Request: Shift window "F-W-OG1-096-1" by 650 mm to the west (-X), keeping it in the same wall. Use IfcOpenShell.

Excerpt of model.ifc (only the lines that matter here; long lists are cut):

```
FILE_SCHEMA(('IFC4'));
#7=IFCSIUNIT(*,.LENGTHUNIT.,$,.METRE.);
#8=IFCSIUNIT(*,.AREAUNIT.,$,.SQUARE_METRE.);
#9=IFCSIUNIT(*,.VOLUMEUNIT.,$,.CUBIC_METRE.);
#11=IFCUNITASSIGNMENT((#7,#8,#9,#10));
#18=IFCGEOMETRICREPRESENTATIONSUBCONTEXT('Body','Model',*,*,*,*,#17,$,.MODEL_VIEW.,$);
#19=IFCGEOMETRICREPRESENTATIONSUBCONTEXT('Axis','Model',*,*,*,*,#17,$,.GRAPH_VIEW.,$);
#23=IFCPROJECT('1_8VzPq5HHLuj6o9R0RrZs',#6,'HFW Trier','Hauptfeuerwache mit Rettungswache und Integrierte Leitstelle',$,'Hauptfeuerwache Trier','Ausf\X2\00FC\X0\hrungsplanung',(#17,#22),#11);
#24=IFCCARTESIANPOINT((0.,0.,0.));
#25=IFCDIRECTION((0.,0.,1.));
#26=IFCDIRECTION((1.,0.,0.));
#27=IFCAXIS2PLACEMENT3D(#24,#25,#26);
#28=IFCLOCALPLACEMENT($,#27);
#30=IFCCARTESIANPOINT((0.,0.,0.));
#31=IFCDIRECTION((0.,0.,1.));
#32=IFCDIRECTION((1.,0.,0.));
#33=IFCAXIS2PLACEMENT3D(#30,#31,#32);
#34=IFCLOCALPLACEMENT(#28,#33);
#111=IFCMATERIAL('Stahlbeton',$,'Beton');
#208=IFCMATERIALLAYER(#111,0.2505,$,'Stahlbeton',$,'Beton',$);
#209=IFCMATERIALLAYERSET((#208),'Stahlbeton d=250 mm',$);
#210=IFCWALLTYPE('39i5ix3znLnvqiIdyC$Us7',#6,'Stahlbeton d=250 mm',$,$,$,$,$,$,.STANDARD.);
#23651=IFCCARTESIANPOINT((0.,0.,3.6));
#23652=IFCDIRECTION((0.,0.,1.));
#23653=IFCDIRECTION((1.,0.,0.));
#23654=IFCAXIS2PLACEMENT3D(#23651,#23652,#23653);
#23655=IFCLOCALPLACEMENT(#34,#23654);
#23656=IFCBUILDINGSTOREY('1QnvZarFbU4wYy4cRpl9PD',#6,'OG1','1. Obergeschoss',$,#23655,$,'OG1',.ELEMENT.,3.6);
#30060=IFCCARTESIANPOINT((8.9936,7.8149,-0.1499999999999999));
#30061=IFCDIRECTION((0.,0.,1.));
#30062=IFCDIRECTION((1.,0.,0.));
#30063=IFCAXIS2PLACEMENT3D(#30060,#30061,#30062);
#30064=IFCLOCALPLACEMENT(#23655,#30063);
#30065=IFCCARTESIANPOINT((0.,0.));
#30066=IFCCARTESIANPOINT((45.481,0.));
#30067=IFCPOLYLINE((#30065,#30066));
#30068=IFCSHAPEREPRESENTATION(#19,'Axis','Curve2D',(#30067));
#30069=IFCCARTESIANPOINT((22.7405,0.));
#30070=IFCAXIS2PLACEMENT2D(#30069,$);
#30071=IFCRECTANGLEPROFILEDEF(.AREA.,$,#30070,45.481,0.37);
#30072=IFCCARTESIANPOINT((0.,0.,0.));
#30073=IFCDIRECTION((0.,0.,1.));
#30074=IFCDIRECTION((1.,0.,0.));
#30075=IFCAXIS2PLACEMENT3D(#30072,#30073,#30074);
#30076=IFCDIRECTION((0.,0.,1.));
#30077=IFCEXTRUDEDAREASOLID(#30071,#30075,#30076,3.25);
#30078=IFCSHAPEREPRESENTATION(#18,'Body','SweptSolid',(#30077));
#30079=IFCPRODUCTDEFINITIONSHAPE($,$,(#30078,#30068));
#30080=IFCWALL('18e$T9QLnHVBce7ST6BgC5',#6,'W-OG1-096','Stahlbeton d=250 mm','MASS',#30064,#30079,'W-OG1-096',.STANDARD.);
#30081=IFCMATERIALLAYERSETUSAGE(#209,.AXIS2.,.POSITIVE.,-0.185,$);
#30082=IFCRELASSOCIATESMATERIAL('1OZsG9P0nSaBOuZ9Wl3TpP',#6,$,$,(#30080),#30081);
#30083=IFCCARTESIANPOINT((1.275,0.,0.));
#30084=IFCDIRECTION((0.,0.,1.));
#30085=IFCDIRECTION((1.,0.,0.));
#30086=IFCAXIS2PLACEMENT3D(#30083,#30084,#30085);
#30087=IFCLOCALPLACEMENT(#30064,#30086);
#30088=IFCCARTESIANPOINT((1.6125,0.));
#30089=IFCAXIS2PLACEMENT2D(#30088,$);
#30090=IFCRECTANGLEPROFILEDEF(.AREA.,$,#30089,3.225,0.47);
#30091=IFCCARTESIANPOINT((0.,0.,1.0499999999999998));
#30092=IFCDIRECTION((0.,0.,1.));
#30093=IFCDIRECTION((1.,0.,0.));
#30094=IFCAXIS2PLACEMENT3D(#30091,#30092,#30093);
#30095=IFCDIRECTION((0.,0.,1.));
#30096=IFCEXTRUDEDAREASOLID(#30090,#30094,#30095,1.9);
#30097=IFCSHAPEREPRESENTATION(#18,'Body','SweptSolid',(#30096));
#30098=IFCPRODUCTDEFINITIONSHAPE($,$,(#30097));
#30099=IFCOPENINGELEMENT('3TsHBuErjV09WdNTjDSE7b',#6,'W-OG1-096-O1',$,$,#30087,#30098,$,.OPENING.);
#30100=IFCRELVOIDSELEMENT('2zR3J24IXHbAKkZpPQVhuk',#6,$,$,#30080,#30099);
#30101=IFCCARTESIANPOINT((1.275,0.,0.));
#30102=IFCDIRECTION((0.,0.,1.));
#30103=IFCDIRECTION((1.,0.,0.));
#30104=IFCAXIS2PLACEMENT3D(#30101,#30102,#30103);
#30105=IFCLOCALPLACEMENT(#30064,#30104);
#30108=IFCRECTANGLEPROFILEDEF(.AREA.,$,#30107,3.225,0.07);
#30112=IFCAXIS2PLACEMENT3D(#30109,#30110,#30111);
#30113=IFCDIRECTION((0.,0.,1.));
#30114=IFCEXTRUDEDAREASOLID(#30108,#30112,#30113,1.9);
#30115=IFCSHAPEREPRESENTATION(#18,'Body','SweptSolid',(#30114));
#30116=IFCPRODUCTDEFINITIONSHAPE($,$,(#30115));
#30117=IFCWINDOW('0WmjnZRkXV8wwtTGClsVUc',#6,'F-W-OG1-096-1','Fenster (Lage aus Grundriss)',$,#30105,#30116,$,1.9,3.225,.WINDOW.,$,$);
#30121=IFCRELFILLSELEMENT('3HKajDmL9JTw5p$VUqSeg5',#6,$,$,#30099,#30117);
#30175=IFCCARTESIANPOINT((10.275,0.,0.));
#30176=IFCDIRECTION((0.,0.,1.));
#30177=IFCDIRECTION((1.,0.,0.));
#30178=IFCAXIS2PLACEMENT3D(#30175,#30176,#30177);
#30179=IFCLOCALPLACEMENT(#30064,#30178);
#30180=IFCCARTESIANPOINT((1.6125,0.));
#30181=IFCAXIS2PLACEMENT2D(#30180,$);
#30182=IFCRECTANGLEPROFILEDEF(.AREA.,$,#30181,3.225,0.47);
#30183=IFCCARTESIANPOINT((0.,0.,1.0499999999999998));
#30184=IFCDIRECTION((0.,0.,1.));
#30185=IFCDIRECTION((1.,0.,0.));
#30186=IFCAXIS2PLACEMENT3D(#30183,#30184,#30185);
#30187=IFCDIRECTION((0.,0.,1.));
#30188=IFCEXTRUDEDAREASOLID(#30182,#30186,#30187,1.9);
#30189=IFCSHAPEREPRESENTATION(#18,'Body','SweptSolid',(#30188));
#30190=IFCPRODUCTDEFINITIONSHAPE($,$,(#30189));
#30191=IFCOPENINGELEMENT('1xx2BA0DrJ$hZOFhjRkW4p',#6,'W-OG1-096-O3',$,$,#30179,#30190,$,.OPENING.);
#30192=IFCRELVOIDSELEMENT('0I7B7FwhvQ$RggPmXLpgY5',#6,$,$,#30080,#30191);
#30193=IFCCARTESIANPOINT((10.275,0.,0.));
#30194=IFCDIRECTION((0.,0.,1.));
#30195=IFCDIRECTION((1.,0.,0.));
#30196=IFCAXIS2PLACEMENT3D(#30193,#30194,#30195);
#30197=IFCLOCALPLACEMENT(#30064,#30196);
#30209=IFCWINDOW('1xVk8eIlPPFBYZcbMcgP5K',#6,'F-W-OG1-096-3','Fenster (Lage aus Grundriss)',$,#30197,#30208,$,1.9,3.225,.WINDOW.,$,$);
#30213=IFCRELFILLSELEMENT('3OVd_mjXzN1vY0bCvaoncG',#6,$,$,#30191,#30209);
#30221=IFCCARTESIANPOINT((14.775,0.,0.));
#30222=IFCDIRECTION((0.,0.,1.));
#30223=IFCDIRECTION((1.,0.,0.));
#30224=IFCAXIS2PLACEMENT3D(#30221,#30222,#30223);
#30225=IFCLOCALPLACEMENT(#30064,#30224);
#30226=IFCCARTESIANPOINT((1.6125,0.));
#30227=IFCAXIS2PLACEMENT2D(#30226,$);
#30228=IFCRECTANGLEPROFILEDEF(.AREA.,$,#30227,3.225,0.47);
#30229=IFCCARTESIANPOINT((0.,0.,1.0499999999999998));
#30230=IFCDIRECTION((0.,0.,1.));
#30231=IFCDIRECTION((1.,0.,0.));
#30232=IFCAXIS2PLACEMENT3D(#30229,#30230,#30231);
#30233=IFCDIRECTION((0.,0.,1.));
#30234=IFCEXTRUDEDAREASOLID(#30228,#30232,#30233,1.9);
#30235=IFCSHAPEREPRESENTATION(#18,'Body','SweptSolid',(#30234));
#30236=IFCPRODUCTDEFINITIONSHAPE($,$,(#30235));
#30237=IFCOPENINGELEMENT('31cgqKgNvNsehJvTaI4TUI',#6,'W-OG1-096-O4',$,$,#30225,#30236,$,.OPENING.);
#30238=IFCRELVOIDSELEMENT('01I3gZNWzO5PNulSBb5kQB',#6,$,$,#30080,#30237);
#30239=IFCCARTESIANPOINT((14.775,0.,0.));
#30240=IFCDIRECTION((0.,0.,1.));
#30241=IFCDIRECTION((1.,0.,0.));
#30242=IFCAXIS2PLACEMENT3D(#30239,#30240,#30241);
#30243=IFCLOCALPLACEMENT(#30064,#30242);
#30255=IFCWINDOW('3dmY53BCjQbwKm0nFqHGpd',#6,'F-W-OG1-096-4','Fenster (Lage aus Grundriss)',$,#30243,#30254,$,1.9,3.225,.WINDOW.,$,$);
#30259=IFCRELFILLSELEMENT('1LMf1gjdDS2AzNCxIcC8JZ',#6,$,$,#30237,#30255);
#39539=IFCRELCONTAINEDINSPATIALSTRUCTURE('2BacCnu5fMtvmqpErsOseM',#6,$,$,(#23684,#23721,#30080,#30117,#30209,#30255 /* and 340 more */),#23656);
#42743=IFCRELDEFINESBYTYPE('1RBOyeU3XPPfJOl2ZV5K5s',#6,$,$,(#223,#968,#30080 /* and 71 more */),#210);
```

```python
import ifcopenshell
import ifcopenshell.api.geometry
import ifcopenshell.util.placement
import ifcopenshell.util.unit

model = ifcopenshell.open("model.ifc")
unit_scale = ifcopenshell.util.unit.calculate_unit_scale(model)

window = model.by_guid("0WmjnZRkXV8wwtTGClsVUc")
opening = window.FillsVoids[0].RelatingOpeningElement
wall = opening.VoidsElements[0].RelatingBuildingElement

wall_matrix = ifcopenshell.util.placement.get_local_placement(wall.ObjectPlacement)
shift = wall_matrix[:3, 0] * -0.65 / unit_scale
before = ifcopenshell.util.placement.get_local_placement(window.ObjectPlacement)[:3, 3].copy()

# The window is not placed relative to its opening, so move both.
for product in (opening, window):
    matrix = ifcopenshell.util.placement.get_local_placement(product.ObjectPlacement)
    matrix[:3, 3] += shift
    ifcopenshell.api.geometry.edit_object_placement(model, product=product, matrix=matrix, is_si=False)

after = ifcopenshell.util.placement.get_local_placement(window.ObjectPlacement)[:3, 3]
print("window moved by", (after - before).round(3) + 0.0)

model.write("model_edited.ifc")
```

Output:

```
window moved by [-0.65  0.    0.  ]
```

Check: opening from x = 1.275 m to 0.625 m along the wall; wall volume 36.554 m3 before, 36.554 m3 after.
